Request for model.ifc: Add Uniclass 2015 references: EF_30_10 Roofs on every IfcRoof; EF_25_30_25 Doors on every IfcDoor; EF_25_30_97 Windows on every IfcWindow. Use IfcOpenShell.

First a look at what the model holds.

```python
import ifcopenshell

model = ifcopenshell.open("model.ifc")
print(model.schema)
print("classifications:", [c.Name for c in model.by_type("IfcClassification")])
for ifc_class in ("IfcDoor", "IfcRoof", "IfcStair", "IfcWall", "IfcWindow"):
    print(ifc_class, len(model.by_type(ifc_class)))
```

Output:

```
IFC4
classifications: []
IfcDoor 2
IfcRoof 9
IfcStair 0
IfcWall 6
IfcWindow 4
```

```python
import ifcopenshell
import ifcopenshell.api.classification

model = ifcopenshell.open("model.ifc")

system = ifcopenshell.api.classification.add_classification(model, classification="Uniclass 2015")

codes = {
    "IfcRoof": ("EF_30_10", "Roofs"),
    "IfcDoor": ("EF_25_30_25", "Doors"),
    "IfcWindow": ("EF_25_30_97", "Windows"),
}
for ifc_class, (code, name) in codes.items():
    products = model.by_type(ifc_class)
    ifcopenshell.api.classification.add_reference(
        model, products=products, classification=system, identification=code, name=name
    )
    print(code, len(products))

model.write("model_updated.ifc")
```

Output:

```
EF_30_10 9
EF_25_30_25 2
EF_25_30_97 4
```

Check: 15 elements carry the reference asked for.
